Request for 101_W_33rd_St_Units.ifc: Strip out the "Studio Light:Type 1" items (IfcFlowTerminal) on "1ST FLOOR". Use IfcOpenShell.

First a look at what the model holds.

```python
import ifcopenshell
import ifcopenshell.util.element

model = ifcopenshell.open("101_W_33rd_St_Units.ifc")
print(model.schema)
storey = next(s for s in model.by_type("IfcBuildingStorey") if s.Name == "1ST FLOOR")
terminals = [e for e in ifcopenshell.util.element.get_decomposition(storey) if e.is_a("IfcFlowTerminal")]
seen = {}
for e in terminals:
    element_type = ifcopenshell.util.element.get_type(e)
    name = element_type.Name if element_type not in (None, e) else None
    seen[name] = seen.get(name, 0) + 1
for name, count in sorted(seen.items(), key=str):
    print(count, "x", name)
```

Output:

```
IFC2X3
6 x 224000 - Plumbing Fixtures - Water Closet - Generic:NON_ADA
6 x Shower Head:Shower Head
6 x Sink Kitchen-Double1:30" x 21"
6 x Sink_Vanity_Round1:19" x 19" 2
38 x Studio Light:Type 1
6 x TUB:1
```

```python
import ifcopenshell
import ifcopenshell.api.root
import ifcopenshell.util.element

model = ifcopenshell.open("101_W_33rd_St_Units.ifc")

storey = next(s for s in model.by_type("IfcBuildingStorey") if s.Name == "1ST FLOOR")
terminals = [e for e in ifcopenshell.util.element.get_decomposition(storey) if e.is_a("IfcFlowTerminal")]
targets = [e for e in terminals if (t := ifcopenshell.util.element.get_type(e)) not in (None, e) and t.Name == "Studio Light:Type 1"]

for e in targets:
    ifcopenshell.api.root.remove_product(model, product=e)
print(len(targets), "removed")

model.write("101_W_33rd_St_Units_v2.ifc")
```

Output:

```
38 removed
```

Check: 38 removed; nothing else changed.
